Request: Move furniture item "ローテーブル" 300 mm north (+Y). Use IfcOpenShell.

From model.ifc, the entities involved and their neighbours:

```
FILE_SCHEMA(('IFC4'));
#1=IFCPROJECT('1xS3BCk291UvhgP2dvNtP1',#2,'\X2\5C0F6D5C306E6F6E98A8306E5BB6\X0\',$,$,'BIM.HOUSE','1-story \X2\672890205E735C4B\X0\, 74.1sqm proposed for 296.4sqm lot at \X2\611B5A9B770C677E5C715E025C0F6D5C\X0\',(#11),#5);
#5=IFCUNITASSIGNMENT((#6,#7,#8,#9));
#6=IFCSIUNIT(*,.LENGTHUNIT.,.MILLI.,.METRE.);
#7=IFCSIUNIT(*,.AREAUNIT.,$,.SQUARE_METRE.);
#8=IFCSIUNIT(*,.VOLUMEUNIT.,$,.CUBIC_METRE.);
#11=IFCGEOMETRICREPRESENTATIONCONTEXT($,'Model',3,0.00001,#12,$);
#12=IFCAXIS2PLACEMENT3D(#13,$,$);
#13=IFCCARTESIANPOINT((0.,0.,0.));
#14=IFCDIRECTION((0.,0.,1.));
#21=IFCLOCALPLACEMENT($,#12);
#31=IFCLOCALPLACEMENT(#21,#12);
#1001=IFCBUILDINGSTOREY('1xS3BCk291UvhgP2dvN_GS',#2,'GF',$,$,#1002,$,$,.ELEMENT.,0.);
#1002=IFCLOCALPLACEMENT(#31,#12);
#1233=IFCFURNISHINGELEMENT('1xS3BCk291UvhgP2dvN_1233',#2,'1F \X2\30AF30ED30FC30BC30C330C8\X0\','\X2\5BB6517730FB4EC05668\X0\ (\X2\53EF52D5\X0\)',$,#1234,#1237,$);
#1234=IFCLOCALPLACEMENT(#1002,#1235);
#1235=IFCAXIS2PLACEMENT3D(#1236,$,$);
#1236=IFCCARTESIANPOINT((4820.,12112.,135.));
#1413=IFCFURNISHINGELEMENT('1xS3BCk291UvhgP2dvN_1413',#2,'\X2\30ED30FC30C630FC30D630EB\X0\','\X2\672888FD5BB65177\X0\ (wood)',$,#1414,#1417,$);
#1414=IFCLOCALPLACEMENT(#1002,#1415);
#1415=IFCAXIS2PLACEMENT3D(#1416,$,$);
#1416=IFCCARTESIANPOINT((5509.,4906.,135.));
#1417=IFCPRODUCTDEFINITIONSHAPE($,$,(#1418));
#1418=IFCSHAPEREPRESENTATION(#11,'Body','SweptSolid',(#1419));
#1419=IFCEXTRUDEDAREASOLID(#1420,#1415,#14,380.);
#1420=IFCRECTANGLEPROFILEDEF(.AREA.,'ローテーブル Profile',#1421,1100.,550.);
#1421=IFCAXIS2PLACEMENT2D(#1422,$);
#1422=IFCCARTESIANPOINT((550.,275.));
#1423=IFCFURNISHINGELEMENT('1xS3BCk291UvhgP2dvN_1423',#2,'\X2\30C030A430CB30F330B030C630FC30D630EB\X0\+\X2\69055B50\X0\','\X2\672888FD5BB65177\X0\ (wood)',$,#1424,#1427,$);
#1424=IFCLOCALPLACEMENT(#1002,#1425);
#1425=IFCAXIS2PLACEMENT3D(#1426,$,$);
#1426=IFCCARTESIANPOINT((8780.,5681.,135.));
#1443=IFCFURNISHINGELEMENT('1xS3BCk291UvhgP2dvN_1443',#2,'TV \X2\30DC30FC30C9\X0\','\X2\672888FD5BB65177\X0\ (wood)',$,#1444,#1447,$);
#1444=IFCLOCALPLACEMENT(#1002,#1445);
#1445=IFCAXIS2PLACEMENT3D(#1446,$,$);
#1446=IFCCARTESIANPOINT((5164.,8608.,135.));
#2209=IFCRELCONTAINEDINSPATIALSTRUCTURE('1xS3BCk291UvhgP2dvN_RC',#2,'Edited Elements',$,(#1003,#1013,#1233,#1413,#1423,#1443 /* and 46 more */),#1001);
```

```python
import ifcopenshell
import ifcopenshell.api.geometry
import ifcopenshell.util.placement
import ifcopenshell.util.unit

model = ifcopenshell.open("model.ifc")
unit_scale = ifcopenshell.util.unit.calculate_unit_scale(model)

item = model.by_guid("1xS3BCk291UvhgP2dvN_1413")
matrix = ifcopenshell.util.placement.get_local_placement(item.ObjectPlacement)
matrix[1, 3] += 0.3 / unit_scale
ifcopenshell.api.geometry.edit_object_placement(model, product=item, matrix=matrix, is_si=False)

print(ifcopenshell.util.placement.get_local_placement(item.ObjectPlacement).round(3) + 0.0)

model.write("model_rev.ifc")
```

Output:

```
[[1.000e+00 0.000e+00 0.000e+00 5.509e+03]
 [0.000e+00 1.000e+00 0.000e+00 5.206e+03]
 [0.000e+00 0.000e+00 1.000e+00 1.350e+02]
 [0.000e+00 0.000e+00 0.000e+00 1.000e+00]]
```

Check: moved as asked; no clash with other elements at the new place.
